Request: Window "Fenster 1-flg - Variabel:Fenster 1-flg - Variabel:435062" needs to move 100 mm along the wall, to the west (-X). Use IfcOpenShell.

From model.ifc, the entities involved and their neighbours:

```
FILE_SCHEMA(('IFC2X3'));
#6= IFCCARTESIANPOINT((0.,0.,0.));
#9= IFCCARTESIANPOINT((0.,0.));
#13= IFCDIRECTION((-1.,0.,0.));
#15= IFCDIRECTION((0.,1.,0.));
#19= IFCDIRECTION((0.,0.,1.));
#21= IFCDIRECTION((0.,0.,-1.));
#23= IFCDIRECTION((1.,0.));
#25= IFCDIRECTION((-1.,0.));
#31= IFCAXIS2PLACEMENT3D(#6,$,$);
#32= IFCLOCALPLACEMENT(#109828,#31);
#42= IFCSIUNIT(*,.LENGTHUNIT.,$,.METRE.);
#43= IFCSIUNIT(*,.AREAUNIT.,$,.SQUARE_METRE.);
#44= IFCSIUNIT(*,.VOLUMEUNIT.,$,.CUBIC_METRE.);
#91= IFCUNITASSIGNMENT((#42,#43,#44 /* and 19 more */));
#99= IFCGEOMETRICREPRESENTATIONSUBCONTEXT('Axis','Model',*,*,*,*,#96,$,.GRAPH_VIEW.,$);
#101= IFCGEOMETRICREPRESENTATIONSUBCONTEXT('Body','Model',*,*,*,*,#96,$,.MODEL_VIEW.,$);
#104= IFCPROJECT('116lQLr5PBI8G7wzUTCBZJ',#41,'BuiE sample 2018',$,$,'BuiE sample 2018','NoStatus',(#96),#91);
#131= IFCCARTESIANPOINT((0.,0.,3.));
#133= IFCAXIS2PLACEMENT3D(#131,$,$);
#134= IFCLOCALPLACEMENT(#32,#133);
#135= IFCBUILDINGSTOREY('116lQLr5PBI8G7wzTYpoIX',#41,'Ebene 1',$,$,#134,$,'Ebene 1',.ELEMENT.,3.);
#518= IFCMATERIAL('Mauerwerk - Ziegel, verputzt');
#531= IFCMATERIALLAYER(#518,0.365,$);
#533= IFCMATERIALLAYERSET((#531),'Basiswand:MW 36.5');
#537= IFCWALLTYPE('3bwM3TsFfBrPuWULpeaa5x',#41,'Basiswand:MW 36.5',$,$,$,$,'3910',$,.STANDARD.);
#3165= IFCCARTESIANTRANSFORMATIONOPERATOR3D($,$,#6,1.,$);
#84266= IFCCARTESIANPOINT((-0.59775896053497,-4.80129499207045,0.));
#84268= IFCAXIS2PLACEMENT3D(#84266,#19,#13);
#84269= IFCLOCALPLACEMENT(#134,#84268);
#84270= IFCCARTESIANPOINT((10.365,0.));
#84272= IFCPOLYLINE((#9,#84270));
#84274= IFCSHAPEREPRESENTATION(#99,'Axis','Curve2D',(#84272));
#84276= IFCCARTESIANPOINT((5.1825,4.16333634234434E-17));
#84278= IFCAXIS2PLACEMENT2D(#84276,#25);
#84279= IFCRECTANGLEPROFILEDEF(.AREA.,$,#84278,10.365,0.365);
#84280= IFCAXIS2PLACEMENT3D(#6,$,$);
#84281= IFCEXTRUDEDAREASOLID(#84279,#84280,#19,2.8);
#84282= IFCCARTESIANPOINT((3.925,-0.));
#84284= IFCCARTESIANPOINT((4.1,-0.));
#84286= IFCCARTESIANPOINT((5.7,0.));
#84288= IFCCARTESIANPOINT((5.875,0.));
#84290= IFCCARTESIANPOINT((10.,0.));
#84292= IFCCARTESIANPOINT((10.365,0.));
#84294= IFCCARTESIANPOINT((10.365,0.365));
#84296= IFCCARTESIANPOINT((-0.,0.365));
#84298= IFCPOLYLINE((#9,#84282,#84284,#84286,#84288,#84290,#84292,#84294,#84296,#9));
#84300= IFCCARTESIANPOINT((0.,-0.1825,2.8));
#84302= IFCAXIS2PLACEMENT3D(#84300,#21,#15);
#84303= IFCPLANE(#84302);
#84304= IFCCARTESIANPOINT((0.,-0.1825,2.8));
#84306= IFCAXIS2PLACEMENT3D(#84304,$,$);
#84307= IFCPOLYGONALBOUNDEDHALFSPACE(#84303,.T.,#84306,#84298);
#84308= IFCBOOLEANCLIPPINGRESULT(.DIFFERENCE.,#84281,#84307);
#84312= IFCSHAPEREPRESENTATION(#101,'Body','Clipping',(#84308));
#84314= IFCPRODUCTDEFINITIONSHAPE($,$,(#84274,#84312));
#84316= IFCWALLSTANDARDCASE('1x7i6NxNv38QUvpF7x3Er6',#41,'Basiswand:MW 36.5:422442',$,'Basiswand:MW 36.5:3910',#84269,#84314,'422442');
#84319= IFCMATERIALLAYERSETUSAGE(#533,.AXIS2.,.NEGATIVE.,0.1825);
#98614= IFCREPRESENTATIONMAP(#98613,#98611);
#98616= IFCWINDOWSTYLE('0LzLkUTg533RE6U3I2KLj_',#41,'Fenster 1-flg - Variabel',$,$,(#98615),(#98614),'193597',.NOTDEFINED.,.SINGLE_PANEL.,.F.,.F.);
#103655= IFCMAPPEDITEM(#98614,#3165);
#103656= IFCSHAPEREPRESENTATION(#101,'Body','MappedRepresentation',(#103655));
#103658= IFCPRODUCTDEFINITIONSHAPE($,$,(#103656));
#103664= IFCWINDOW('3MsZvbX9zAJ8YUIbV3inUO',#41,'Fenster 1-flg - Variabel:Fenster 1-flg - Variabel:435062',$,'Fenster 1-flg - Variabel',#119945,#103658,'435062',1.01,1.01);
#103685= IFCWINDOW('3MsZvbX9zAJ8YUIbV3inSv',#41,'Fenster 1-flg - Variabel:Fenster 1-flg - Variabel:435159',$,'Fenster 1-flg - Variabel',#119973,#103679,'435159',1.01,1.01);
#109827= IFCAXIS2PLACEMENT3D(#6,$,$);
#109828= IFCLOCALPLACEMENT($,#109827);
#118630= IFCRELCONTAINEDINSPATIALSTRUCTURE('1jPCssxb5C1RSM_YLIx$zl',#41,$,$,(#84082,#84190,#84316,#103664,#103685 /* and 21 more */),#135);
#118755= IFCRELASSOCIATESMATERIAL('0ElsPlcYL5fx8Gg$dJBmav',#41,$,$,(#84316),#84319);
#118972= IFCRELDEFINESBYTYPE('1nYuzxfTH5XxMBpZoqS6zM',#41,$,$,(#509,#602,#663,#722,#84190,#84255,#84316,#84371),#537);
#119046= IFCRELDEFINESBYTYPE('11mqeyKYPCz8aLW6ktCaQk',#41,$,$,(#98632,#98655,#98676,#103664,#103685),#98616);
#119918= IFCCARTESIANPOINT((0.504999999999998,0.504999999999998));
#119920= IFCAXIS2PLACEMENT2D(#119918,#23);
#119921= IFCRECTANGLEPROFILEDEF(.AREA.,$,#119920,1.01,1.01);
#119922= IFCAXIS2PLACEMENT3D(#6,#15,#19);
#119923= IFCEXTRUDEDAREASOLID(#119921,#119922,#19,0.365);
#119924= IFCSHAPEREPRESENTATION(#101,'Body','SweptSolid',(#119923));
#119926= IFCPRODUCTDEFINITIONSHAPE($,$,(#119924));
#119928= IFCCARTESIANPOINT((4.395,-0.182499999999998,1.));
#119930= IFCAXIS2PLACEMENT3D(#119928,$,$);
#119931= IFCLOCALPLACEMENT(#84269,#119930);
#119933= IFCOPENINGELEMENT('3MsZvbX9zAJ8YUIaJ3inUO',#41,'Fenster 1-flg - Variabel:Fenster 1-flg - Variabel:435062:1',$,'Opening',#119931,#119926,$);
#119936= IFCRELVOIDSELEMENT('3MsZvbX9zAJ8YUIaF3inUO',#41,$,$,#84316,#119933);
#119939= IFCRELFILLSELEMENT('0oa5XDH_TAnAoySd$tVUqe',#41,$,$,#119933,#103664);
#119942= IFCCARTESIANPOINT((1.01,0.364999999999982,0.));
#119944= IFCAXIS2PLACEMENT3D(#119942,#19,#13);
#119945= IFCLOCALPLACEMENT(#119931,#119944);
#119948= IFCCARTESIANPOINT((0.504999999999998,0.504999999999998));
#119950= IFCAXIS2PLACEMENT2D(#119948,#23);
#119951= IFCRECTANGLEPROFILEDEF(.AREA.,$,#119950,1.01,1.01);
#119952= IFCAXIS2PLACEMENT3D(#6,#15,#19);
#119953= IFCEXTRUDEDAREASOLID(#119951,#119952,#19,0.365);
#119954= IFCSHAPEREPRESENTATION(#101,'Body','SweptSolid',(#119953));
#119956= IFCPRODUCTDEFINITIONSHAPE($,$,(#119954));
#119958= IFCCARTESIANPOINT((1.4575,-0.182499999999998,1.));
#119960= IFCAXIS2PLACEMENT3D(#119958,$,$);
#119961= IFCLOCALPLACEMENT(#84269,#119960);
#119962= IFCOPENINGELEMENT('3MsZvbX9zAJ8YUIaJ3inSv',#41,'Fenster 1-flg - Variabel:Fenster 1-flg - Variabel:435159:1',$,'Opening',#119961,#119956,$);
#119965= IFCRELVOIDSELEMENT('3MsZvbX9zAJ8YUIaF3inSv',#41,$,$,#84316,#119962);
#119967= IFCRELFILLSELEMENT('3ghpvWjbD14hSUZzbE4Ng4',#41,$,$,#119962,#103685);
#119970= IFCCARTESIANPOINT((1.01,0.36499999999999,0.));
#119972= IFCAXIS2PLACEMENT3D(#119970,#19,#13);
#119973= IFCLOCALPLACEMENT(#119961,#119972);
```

```python
import ifcopenshell
import ifcopenshell.api.geometry
import ifcopenshell.util.placement

model = ifcopenshell.open("model.ifc")

window = model.by_guid("3MsZvbX9zAJ8YUIbV3inUO")
opening = window.FillsVoids[0].RelatingOpeningElement
wall = opening.VoidsElements[0].RelatingBuildingElement

wall_matrix = ifcopenshell.util.placement.get_local_placement(wall.ObjectPlacement)
shift = wall_matrix[:3, 0] * 0.1
before = ifcopenshell.util.placement.get_local_placement(window.ObjectPlacement)[:3, 3].copy()

# The window is placed relative to its opening, so it follows when the opening moves.
matrix = ifcopenshell.util.placement.get_local_placement(opening.ObjectPlacement)
matrix[:3, 3] += shift
ifcopenshell.api.geometry.edit_object_placement(
    model, product=opening, matrix=matrix, is_si=False, should_transform_children=True
)

after = ifcopenshell.util.placement.get_local_placement(window.ObjectPlacement)[:3, 3]
print("window moved by", (after - before).round(3) + 0.0)

model.write("model_v2.ifc")
```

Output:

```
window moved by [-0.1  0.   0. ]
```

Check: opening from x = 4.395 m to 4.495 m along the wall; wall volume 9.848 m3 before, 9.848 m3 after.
